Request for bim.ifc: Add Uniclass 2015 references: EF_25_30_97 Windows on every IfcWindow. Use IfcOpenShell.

First a look at what the model holds.

```python
import ifcopenshell

model = ifcopenshell.open("bim.ifc")
print(model.schema)
print("classifications:", [c.Name for c in model.by_type("IfcClassification")])
for ifc_class in ("IfcDoor", "IfcRoof", "IfcStair", "IfcWall", "IfcWindow"):
    print(ifc_class, len(model.by_type(ifc_class)))
```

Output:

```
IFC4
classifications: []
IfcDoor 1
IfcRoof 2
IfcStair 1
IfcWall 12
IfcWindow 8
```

```python
import ifcopenshell
import ifcopenshell.api.classification

model = ifcopenshell.open("bim.ifc")

system = ifcopenshell.api.classification.add_classification(model, classification="Uniclass 2015")

codes = {
    "IfcWindow": ("EF_25_30_97", "Windows"),
}
for ifc_class, (code, name) in codes.items():
    products = model.by_type(ifc_class)
    ifcopenshell.api.classification.add_reference(
        model, products=products, classification=system, identification=code, name=name
    )
    print(code, len(products))

model.write("bim_edited.ifc")
```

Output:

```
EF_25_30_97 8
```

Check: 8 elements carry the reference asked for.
